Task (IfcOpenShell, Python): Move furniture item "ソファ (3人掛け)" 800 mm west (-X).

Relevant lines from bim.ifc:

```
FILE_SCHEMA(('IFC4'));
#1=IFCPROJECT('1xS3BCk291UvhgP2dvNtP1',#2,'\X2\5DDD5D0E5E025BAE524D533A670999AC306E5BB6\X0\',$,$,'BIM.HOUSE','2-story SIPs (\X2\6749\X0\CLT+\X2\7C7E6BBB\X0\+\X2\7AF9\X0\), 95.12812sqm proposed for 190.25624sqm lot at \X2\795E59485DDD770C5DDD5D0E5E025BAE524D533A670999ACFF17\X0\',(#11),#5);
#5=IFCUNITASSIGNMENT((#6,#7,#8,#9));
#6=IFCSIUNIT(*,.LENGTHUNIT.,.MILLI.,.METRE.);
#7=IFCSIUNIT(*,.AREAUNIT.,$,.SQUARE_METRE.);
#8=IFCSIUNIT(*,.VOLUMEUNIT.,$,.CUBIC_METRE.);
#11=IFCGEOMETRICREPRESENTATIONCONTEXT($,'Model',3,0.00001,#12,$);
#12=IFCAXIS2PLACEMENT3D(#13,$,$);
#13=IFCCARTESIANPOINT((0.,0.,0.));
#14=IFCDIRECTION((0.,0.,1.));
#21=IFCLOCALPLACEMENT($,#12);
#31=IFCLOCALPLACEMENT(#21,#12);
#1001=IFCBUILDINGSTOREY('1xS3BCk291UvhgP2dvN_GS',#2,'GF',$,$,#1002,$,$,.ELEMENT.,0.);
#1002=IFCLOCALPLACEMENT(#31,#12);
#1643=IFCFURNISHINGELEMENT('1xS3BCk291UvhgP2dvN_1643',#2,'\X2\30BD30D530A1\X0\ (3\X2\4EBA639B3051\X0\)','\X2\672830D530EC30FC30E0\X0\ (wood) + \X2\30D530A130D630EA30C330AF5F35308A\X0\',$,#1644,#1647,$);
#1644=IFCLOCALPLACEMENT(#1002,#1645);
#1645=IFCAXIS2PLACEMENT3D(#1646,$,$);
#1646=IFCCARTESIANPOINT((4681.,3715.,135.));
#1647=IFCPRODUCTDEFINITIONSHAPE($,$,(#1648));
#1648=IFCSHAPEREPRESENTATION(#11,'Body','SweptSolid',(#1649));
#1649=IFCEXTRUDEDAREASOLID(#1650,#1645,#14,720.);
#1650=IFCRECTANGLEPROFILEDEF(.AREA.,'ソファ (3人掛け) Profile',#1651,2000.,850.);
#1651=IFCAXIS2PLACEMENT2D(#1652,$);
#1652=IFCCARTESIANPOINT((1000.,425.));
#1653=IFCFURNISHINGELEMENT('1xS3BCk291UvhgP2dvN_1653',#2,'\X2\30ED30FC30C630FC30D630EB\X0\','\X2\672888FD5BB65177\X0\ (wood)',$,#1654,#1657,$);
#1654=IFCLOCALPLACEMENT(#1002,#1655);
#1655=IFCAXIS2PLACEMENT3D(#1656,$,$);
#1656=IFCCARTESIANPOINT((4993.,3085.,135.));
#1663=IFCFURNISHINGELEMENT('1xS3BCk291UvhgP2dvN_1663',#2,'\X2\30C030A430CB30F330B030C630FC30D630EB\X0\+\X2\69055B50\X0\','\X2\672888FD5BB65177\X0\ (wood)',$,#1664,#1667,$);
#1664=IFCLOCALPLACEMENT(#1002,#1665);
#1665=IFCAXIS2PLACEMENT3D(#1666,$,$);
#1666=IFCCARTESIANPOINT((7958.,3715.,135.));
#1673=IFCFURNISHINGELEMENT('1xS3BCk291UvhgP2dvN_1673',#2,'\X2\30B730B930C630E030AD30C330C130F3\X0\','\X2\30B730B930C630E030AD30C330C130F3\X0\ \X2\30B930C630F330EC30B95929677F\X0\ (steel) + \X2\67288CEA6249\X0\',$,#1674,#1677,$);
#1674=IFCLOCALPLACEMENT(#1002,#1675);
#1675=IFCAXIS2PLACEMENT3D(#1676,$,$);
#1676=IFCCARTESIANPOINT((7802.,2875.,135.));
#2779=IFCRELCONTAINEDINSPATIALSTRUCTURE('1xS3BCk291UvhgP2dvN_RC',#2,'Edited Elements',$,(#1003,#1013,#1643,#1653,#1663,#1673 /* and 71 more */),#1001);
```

```python
import ifcopenshell
import ifcopenshell.api.geometry
import ifcopenshell.util.placement

model = ifcopenshell.open("bim.ifc")

item = model.by_guid("1xS3BCk291UvhgP2dvN_1643")
matrix = ifcopenshell.util.placement.get_local_placement(item.ObjectPlacement)
matrix[0, 3] -= 800.0
ifcopenshell.api.geometry.edit_object_placement(model, product=item, matrix=matrix, is_si=False)

print(ifcopenshell.util.placement.get_local_placement(item.ObjectPlacement).round(3) + 0.0)

model.write("bim_rev.ifc")
```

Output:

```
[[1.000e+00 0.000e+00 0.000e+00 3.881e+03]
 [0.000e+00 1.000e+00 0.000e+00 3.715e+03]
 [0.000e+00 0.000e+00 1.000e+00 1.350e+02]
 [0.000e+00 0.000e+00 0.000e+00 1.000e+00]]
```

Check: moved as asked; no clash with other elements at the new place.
